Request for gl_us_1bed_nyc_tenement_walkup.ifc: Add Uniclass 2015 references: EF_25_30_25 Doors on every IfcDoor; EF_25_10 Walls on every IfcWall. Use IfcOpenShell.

First a look at what the model holds.

```python
import ifcopenshell

model = ifcopenshell.open("gl_us_1bed_nyc_tenement_walkup.ifc")
print(model.schema)
print("classifications:", [c.Name for c in model.by_type("IfcClassification")])
for ifc_class in ("IfcDoor", "IfcRoof", "IfcStair", "IfcWall", "IfcWindow"):
    print(ifc_class, len(model.by_type(ifc_class)))
```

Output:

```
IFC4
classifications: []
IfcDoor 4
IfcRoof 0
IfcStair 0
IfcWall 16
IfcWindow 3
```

```python
import ifcopenshell
import ifcopenshell.api.classification

model = ifcopenshell.open("gl_us_1bed_nyc_tenement_walkup.ifc")

system = ifcopenshell.api.classification.add_classification(model, classification="Uniclass 2015")

codes = {
    "IfcDoor": ("EF_25_30_25", "Doors"),
    "IfcWall": ("EF_25_10", "Walls"),
}
for ifc_class, (code, name) in codes.items():
    products = model.by_type(ifc_class)
    ifcopenshell.api.classification.add_reference(
        model, products=products, classification=system, identification=code, name=name
    )
    print(code, len(products))

model.write("gl_us_1bed_nyc_tenement_walkup_edited.ifc")
```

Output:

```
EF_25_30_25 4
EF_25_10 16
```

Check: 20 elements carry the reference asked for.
